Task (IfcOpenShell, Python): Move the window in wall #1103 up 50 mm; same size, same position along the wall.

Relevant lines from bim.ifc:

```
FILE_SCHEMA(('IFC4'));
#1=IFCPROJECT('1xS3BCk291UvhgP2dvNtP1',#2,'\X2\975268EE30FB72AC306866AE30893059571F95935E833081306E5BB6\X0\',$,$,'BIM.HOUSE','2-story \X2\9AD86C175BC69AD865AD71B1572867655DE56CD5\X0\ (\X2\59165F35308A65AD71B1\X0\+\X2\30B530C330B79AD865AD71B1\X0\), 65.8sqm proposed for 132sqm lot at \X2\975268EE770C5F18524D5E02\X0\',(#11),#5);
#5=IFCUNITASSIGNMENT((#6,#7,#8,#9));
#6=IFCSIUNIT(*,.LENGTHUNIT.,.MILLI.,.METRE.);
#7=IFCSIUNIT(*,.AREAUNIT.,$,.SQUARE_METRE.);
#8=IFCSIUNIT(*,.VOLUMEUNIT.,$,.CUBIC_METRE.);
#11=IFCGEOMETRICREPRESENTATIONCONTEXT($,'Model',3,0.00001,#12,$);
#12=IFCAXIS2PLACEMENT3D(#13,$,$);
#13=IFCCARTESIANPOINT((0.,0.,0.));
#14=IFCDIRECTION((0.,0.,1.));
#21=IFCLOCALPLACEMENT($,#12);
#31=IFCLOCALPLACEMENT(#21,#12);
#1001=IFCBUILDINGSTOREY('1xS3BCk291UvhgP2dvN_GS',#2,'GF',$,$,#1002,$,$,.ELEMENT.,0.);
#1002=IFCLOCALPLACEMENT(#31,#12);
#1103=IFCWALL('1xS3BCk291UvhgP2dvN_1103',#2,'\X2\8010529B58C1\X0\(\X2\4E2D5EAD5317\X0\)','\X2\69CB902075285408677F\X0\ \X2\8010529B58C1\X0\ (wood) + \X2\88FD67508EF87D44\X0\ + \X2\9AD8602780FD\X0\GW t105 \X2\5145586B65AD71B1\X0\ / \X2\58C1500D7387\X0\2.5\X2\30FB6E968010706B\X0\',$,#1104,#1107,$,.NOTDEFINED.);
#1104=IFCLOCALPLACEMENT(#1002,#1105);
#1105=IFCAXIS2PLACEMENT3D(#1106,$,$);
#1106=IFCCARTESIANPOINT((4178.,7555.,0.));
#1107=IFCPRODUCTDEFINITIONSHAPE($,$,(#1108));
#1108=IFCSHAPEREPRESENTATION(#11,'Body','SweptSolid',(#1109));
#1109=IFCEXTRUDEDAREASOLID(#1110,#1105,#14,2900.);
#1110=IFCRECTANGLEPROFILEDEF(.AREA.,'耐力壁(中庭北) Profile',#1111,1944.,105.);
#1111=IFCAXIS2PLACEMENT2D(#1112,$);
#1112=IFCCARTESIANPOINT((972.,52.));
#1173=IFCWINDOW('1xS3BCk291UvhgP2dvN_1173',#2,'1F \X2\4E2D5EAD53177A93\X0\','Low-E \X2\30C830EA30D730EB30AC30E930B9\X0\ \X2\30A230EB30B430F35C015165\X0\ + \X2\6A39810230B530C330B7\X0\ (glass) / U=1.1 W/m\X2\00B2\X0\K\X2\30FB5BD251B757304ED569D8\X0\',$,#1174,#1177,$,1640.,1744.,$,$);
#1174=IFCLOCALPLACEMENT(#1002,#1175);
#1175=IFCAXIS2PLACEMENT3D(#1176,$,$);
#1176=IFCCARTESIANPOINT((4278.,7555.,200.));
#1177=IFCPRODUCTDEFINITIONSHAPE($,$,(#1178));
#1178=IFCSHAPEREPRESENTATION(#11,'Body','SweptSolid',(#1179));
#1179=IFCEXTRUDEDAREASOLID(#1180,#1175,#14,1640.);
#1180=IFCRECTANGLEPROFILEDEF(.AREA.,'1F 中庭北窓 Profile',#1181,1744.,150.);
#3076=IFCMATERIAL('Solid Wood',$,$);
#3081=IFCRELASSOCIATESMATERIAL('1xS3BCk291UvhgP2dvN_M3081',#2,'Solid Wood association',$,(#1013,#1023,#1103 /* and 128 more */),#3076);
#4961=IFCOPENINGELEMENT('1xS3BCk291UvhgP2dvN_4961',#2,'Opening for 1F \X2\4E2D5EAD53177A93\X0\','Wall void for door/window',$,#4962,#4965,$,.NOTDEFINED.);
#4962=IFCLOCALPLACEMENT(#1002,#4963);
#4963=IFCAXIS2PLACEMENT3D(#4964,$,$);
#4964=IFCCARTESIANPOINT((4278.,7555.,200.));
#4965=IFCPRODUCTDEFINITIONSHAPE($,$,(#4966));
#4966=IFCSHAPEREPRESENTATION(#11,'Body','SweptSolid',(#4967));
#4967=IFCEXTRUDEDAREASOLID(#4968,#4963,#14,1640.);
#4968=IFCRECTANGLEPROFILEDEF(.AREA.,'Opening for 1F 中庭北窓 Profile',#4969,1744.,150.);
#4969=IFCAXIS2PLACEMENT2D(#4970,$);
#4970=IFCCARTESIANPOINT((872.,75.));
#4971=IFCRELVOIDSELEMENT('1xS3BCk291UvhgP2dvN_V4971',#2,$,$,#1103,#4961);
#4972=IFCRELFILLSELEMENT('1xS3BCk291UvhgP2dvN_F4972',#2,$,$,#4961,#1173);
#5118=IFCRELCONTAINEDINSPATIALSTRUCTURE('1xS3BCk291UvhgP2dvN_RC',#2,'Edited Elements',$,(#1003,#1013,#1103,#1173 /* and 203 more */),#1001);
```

```python
import numpy as np
import ifcopenshell
import ifcopenshell.api.geometry
import ifcopenshell.util.placement
import ifcopenshell.util.unit

model = ifcopenshell.open("bim.ifc")
unit_scale = ifcopenshell.util.unit.calculate_unit_scale(model)

window = model.by_id(1173)
opening = window.FillsVoids[0].RelatingOpeningElement
dz = 50.0

shift = np.array([0.0, 0.0, dz])
# The window is not placed relative to its opening, so move both.
for product in (opening, window):
    matrix = ifcopenshell.util.placement.get_local_placement(product.ObjectPlacement)
    matrix[:3, 3] += shift
    ifcopenshell.api.geometry.edit_object_placement(model, product=product, matrix=matrix, is_si=False)

print(f"moved by {dz * unit_scale:+.3f} m")

model.write("bim_v2.ifc")
```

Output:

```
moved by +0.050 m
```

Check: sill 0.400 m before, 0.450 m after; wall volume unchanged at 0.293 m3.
